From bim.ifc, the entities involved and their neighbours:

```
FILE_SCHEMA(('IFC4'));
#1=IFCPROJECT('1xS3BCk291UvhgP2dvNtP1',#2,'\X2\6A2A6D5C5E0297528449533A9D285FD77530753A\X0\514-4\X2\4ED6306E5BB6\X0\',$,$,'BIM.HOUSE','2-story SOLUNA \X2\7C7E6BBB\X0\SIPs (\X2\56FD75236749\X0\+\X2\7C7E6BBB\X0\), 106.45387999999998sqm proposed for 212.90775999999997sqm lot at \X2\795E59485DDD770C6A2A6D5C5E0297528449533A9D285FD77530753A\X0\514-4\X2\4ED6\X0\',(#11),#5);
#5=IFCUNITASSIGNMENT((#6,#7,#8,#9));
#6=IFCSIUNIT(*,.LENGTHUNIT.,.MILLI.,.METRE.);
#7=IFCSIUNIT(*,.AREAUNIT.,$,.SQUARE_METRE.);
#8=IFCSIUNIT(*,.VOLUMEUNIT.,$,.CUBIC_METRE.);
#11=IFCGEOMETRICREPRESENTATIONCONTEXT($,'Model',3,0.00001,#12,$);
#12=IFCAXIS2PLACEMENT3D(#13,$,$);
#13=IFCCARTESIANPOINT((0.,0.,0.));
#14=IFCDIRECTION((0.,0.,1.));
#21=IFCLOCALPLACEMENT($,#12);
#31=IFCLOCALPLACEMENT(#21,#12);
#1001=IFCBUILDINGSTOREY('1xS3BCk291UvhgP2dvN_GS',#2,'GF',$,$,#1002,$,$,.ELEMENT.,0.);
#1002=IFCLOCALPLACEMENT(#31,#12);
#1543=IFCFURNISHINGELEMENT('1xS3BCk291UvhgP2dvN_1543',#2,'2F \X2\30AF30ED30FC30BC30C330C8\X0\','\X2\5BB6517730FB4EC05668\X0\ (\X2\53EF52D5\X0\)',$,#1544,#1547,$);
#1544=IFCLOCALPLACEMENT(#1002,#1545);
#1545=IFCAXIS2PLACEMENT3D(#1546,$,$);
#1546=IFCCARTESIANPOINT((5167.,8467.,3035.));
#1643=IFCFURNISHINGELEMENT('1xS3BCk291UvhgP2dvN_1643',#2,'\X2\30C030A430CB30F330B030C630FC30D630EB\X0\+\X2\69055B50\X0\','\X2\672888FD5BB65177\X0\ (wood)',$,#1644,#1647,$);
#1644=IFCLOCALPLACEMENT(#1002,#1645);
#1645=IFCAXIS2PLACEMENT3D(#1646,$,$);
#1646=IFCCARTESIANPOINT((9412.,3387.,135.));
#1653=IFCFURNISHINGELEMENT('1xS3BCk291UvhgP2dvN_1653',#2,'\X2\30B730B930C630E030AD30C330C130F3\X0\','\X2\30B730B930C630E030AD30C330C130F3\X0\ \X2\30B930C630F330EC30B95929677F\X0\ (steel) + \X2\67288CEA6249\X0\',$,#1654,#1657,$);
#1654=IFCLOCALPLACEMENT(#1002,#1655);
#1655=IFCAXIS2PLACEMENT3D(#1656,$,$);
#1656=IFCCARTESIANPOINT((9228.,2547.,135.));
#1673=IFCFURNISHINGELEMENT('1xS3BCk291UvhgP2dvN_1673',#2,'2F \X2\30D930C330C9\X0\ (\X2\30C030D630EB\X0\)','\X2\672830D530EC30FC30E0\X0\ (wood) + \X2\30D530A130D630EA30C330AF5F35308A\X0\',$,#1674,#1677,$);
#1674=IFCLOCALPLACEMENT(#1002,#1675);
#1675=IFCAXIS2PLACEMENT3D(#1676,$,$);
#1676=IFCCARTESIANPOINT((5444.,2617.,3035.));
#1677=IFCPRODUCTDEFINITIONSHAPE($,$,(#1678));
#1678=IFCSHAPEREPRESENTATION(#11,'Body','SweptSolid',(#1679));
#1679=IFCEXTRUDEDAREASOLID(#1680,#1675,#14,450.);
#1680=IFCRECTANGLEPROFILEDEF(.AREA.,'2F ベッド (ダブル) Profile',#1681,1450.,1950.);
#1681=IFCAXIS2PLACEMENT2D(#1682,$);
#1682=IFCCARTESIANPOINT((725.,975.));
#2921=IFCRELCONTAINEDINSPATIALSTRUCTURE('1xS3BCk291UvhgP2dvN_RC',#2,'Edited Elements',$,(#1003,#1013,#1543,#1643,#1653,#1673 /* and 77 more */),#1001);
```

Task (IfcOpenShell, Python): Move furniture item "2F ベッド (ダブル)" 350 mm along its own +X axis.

```python
import ifcopenshell
import ifcopenshell.api.geometry
import ifcopenshell.util.placement
import ifcopenshell.util.unit

model = ifcopenshell.open("bim.ifc")
unit_scale = ifcopenshell.util.unit.calculate_unit_scale(model)

item = model.by_guid("1xS3BCk291UvhgP2dvN_1673")
matrix = ifcopenshell.util.placement.get_local_placement(item.ObjectPlacement)
matrix[:3, 3] += matrix[:3, 0] * 0.35 / unit_scale
ifcopenshell.api.geometry.edit_object_placement(model, product=item, matrix=matrix, is_si=False)

print(ifcopenshell.util.placement.get_local_placement(item.ObjectPlacement).round(3) + 0.0)

model.write("bim-out.ifc")
```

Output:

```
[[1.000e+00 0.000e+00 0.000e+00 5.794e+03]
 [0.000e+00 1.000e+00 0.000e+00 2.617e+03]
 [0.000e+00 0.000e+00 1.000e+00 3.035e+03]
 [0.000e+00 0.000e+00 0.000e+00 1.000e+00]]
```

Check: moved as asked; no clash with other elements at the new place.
